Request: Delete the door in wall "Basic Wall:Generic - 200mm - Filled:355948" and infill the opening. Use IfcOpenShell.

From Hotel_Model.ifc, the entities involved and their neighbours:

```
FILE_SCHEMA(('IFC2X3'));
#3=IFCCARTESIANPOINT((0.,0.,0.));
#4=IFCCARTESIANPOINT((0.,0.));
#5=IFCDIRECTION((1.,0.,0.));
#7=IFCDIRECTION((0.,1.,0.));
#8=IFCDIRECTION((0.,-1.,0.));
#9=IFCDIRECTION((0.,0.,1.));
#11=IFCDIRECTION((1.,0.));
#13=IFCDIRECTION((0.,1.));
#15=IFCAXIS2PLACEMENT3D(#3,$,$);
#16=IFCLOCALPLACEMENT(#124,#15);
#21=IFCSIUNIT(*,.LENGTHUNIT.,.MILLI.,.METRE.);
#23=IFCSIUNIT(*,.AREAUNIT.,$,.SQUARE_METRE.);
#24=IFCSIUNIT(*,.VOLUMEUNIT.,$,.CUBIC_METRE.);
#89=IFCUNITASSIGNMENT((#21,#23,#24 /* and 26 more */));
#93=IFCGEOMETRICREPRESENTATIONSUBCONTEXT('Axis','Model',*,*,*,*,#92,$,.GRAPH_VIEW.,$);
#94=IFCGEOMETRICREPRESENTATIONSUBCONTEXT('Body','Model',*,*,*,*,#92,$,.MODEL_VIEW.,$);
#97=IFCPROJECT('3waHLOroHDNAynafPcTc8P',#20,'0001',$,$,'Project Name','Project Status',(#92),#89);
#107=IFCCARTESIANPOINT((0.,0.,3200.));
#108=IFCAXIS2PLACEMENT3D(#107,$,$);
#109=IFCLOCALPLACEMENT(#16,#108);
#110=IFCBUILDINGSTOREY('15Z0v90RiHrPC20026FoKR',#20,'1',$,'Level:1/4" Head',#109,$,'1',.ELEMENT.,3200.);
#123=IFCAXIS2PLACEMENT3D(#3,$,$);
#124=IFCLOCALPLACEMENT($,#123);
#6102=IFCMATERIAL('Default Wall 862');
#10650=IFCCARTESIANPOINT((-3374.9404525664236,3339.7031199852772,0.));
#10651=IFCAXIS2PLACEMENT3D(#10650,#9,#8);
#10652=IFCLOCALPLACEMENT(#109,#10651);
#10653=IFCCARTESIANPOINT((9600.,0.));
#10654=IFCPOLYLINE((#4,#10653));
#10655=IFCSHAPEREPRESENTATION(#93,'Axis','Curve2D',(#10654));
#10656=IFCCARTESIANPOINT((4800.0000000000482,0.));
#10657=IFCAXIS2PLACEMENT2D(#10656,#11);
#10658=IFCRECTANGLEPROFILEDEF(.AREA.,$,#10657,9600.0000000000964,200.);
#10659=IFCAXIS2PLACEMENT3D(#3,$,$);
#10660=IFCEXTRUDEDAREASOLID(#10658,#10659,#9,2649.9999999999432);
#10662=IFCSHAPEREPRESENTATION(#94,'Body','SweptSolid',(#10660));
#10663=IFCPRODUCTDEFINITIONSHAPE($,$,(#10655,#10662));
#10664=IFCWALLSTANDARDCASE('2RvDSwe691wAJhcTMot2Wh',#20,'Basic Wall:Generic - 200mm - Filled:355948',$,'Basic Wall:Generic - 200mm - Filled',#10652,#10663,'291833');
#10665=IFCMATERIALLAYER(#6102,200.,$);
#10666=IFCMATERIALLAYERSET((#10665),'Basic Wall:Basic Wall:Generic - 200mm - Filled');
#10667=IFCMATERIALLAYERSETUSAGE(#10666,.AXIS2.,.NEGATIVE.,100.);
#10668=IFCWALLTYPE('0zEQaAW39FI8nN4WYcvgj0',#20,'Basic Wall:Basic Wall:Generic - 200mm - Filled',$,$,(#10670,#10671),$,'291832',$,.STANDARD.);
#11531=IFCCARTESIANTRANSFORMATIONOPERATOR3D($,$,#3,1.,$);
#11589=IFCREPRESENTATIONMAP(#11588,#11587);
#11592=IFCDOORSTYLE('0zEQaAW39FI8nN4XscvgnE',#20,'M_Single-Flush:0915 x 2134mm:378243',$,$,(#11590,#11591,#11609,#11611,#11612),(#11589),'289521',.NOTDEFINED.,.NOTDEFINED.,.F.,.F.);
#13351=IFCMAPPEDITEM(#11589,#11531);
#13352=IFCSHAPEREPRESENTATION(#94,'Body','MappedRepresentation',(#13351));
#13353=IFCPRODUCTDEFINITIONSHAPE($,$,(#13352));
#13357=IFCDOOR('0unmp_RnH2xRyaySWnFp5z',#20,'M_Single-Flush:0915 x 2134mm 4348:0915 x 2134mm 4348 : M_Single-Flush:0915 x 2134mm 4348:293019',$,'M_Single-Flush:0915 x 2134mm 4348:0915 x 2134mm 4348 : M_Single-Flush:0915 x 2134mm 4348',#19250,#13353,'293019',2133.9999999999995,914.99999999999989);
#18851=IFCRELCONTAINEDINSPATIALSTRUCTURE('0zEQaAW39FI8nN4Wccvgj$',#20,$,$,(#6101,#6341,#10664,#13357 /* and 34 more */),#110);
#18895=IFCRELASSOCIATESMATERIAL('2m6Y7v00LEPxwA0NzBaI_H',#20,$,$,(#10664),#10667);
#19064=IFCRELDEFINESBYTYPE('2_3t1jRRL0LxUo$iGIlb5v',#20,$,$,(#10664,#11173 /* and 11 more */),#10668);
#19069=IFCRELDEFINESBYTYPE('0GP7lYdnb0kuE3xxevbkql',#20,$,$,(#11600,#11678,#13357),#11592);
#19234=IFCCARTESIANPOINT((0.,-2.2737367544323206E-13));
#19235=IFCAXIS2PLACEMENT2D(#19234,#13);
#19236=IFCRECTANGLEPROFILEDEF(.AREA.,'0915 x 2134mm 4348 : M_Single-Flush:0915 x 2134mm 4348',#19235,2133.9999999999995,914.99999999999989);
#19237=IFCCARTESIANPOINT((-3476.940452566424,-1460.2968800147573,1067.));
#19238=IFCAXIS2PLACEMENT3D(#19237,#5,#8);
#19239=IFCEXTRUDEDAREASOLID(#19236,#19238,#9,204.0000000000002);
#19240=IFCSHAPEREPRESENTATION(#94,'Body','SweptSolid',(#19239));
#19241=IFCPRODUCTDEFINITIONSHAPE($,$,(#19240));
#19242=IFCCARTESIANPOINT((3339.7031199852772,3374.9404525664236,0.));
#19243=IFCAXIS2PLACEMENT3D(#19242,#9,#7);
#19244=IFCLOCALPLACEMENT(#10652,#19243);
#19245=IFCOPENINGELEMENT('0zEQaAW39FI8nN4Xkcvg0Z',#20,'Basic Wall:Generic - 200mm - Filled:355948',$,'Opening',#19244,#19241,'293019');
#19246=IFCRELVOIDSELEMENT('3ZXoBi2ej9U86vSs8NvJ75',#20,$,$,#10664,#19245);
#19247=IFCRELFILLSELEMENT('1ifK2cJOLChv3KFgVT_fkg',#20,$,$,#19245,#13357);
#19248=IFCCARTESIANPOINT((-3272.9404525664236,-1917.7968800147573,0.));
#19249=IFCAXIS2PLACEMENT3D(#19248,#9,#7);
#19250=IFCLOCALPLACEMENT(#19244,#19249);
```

```python
import ifcopenshell
import ifcopenshell.api.feature
import ifcopenshell.api.root
import ifcopenshell.geom
import ifcopenshell.util.shape

model = ifcopenshell.open("Hotel_Model.ifc")
settings = ifcopenshell.geom.settings()


def volume(element):
    """Net volume in cubic metres, openings subtracted."""
    shape = ifcopenshell.geom.create_shape(settings, element)
    return ifcopenshell.util.shape.get_volume(shape.geometry)


door = model.by_id(13357)
opening = door.FillsVoids[0].RelatingOpeningElement
wall = opening.VoidsElements[0].RelatingBuildingElement
before = volume(wall)

ifcopenshell.api.root.remove_product(model, product=door)
ifcopenshell.api.feature.remove_feature(model, feature=opening)

after = volume(wall)

print(f"wall volume {before:.3f} -> {after:.3f} m3")

model.write("Hotel_Model_updated.ifc")
```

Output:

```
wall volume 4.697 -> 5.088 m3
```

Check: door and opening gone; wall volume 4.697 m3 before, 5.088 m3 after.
